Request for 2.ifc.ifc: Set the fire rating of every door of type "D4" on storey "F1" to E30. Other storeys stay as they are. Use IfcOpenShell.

First a look at what the model holds.

```python
import ifcopenshell
import ifcopenshell.util.element

model = ifcopenshell.open("2.ifc.ifc")
print(model.schema)
storey = next(s for s in model.by_type("IfcBuildingStorey") if s.Name == "F1")
doors = [e for e in ifcopenshell.util.element.get_decomposition(storey) if e.is_a("IfcDoor")]
seen = {}
for e in doors:
    element_type = ifcopenshell.util.element.get_type(e)
    key = (element_type.Name if element_type != e and element_type else None, ifcopenshell.util.element.get_pset(e, "Pset_DoorCommon", "FireRating"))
    seen[key] = seen.get(key, 0) + 1
for (name, value), count in sorted(seen.items(), key=str):
    print(count, "x", name, "|", value)
```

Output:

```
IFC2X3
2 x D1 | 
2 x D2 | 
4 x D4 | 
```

```python
import ifcopenshell
import ifcopenshell.api.pset
import ifcopenshell.util.element

model = ifcopenshell.open("2.ifc.ifc")

storey = next(s for s in model.by_type("IfcBuildingStorey") if s.Name == "F1")
doors = [e for e in ifcopenshell.util.element.get_decomposition(storey) if e.is_a("IfcDoor")]

count = 0
for e in doors:
    element_type = ifcopenshell.util.element.get_type(e)
    if element_type in (None, e) or element_type.Name != "D4":
        continue
    # add_pset returns the element's existing set when there is one.
    pset = ifcopenshell.api.pset.add_pset(model, product=e, name="Pset_DoorCommon")
    ifcopenshell.api.pset.edit_pset(model, pset=pset, properties={"FireRating": "E30"})
    count += 1

print(count, "doors updated")

model.write("2.ifc_updated.ifc")
```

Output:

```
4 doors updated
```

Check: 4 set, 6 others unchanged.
